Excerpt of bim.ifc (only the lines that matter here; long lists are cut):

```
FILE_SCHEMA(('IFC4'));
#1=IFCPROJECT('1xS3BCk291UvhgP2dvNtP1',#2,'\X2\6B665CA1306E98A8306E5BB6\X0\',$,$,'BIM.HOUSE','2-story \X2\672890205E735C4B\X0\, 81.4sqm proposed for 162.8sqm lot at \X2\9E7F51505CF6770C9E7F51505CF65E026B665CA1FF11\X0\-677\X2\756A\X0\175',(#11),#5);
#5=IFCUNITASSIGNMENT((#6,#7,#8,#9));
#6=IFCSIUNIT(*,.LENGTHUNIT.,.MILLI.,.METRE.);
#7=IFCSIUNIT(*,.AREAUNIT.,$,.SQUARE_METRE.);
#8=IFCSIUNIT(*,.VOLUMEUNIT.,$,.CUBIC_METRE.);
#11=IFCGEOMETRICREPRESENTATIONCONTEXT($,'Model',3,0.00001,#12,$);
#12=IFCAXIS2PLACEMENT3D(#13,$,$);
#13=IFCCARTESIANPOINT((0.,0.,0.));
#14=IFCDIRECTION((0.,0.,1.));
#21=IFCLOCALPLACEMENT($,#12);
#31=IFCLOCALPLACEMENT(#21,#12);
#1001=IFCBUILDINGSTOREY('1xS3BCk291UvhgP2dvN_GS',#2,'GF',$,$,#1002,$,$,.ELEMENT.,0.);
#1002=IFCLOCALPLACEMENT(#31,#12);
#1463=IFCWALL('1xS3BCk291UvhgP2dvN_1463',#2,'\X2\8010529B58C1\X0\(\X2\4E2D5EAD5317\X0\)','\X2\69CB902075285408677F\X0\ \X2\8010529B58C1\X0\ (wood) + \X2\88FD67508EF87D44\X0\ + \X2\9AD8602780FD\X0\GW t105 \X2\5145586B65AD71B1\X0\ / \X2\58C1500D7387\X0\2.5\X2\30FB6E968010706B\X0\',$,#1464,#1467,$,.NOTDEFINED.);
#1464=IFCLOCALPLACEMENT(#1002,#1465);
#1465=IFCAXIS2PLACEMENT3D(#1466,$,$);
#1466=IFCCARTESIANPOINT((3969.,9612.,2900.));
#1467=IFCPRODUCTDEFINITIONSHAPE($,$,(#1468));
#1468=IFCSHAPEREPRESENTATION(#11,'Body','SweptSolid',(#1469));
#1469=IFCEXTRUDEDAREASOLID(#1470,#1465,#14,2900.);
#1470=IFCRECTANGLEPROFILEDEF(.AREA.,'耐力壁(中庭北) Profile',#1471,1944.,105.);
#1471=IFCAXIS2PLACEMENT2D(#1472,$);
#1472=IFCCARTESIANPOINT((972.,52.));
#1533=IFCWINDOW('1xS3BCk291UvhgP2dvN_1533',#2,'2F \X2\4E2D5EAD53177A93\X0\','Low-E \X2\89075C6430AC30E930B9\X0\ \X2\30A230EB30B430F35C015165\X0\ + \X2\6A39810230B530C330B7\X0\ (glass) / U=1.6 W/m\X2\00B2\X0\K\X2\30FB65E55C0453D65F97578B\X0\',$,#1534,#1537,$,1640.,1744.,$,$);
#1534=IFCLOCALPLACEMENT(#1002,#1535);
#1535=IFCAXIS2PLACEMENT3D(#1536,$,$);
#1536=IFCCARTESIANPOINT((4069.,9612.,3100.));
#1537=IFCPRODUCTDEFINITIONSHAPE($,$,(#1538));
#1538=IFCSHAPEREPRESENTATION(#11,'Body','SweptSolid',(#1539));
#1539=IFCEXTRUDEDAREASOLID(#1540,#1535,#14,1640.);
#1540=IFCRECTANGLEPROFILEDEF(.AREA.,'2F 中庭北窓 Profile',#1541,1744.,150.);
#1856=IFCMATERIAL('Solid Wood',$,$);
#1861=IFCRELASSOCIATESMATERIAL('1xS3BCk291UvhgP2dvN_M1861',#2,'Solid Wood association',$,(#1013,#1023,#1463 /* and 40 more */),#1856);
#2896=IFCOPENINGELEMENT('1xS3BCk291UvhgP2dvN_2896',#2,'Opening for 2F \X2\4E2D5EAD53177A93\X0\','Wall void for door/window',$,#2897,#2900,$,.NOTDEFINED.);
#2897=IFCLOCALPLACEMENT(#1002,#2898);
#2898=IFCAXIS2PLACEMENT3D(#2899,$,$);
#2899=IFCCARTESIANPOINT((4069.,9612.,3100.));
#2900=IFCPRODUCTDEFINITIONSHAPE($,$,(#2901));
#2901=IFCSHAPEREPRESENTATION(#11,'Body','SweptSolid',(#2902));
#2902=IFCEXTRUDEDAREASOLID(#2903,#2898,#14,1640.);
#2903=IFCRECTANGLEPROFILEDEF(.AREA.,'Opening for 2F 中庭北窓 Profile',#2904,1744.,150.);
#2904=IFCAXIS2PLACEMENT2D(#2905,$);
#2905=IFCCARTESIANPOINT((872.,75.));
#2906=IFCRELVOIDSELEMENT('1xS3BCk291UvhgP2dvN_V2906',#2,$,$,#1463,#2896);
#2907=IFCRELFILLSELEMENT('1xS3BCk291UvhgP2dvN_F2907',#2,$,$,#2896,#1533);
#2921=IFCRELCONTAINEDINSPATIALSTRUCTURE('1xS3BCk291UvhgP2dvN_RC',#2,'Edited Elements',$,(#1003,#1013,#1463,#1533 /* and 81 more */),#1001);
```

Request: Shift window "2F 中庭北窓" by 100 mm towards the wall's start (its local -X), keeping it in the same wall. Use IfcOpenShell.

```python
import ifcopenshell
import ifcopenshell.api.geometry
import ifcopenshell.util.placement
import ifcopenshell.util.unit

model = ifcopenshell.open("bim.ifc")
unit_scale = ifcopenshell.util.unit.calculate_unit_scale(model)

window = model.by_guid("1xS3BCk291UvhgP2dvN_1533")
opening = window.FillsVoids[0].RelatingOpeningElement
wall = opening.VoidsElements[0].RelatingBuildingElement

wall_matrix = ifcopenshell.util.placement.get_local_placement(wall.ObjectPlacement)
shift = wall_matrix[:3, 0] * -0.1 / unit_scale
before = ifcopenshell.util.placement.get_local_placement(window.ObjectPlacement)[:3, 3].copy()

# The window is not placed relative to its opening, so move both.
for product in (opening, window):
    matrix = ifcopenshell.util.placement.get_local_placement(product.ObjectPlacement)
    matrix[:3, 3] += shift
    ifcopenshell.api.geometry.edit_object_placement(model, product=product, matrix=matrix, is_si=False)

after = ifcopenshell.util.placement.get_local_placement(window.ObjectPlacement)[:3, 3]
print("window moved by", (after - before).round(3) + 0.0)

model.write("bim_updated.ifc")
```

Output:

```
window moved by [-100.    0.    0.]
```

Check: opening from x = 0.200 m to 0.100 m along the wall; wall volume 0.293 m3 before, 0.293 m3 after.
